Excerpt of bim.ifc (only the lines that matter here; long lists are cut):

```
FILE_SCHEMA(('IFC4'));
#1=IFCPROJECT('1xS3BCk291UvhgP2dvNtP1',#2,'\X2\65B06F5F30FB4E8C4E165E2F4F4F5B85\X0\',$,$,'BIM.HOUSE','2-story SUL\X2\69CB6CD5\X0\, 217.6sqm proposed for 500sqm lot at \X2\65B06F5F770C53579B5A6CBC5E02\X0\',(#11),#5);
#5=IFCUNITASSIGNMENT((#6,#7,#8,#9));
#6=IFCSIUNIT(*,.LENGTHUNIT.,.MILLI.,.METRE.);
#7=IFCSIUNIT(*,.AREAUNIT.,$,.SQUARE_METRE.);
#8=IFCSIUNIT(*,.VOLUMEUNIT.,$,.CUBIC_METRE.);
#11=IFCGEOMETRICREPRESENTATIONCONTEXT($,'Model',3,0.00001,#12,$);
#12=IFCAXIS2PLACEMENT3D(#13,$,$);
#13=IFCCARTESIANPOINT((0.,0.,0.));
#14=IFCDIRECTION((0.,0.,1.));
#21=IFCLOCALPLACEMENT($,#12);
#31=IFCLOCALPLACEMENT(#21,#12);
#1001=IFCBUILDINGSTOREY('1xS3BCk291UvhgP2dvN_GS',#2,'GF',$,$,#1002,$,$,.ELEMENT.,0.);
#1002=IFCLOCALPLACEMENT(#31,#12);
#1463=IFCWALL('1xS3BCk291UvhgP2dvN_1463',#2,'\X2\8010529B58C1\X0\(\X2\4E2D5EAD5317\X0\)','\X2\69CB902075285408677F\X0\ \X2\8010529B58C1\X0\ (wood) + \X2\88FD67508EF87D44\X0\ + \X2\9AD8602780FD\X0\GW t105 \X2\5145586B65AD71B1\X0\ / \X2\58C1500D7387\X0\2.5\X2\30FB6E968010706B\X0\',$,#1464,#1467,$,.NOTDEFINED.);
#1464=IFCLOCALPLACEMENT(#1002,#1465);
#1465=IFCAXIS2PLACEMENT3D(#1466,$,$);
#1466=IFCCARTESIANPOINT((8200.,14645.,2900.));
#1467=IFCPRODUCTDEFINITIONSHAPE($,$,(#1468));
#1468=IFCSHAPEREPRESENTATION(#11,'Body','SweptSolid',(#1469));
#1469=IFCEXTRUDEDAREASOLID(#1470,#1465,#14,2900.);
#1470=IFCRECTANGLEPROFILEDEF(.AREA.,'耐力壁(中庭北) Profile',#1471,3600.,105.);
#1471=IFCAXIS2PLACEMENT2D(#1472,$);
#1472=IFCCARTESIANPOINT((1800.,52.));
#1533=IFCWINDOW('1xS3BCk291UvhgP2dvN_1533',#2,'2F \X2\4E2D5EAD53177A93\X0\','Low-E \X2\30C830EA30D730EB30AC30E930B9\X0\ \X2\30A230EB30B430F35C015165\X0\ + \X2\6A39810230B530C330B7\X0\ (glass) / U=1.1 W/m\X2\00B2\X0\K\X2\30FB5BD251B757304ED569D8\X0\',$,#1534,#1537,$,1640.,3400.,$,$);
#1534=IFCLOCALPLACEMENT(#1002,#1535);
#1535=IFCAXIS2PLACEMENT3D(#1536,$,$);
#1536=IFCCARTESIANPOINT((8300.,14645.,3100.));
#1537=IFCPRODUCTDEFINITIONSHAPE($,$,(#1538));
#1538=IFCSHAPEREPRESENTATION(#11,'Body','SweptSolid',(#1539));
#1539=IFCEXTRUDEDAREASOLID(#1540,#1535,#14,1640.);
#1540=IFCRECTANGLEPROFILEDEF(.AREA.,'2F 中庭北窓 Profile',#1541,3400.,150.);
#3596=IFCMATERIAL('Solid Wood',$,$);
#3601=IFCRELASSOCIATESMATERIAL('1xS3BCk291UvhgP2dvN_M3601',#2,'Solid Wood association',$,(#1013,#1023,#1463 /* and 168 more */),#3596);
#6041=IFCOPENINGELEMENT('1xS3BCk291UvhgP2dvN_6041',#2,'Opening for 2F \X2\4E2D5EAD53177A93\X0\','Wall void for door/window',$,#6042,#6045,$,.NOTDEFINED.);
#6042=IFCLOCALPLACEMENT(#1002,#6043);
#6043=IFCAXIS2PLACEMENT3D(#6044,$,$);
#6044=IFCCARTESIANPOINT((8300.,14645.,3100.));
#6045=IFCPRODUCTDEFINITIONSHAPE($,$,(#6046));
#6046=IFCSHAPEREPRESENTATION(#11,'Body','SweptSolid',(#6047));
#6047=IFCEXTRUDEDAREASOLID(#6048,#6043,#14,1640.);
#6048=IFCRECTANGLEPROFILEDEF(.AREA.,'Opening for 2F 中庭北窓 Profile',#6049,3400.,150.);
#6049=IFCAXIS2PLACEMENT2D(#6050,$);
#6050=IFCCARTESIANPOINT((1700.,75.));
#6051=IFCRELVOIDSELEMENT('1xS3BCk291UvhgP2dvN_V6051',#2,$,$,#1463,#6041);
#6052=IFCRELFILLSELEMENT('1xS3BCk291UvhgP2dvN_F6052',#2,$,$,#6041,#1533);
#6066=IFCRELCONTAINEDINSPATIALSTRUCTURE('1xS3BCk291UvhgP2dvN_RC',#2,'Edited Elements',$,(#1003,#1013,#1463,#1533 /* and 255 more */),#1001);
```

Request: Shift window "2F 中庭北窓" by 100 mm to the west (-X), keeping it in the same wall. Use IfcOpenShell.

```python
import ifcopenshell
import ifcopenshell.api.geometry
import ifcopenshell.util.placement
import ifcopenshell.util.unit

model = ifcopenshell.open("bim.ifc")
unit_scale = ifcopenshell.util.unit.calculate_unit_scale(model)

window = model.by_id(1533)
opening = window.FillsVoids[0].RelatingOpeningElement
wall = opening.VoidsElements[0].RelatingBuildingElement

wall_matrix = ifcopenshell.util.placement.get_local_placement(wall.ObjectPlacement)
shift = wall_matrix[:3, 0] * -0.1 / unit_scale
before = ifcopenshell.util.placement.get_local_placement(window.ObjectPlacement)[:3, 3].copy()

# The window is not placed relative to its opening, so move both.
for product in (opening, window):
    matrix = ifcopenshell.util.placement.get_local_placement(product.ObjectPlacement)
    matrix[:3, 3] += shift
    ifcopenshell.api.geometry.edit_object_placement(model, product=product, matrix=matrix, is_si=False)

after = ifcopenshell.util.placement.get_local_placement(window.ObjectPlacement)[:3, 3]
print("window moved by", (after - before).round(3) + 0.0)

model.write("bim-out.ifc")
```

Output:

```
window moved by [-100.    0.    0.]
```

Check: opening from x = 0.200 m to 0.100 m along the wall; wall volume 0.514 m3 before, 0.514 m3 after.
